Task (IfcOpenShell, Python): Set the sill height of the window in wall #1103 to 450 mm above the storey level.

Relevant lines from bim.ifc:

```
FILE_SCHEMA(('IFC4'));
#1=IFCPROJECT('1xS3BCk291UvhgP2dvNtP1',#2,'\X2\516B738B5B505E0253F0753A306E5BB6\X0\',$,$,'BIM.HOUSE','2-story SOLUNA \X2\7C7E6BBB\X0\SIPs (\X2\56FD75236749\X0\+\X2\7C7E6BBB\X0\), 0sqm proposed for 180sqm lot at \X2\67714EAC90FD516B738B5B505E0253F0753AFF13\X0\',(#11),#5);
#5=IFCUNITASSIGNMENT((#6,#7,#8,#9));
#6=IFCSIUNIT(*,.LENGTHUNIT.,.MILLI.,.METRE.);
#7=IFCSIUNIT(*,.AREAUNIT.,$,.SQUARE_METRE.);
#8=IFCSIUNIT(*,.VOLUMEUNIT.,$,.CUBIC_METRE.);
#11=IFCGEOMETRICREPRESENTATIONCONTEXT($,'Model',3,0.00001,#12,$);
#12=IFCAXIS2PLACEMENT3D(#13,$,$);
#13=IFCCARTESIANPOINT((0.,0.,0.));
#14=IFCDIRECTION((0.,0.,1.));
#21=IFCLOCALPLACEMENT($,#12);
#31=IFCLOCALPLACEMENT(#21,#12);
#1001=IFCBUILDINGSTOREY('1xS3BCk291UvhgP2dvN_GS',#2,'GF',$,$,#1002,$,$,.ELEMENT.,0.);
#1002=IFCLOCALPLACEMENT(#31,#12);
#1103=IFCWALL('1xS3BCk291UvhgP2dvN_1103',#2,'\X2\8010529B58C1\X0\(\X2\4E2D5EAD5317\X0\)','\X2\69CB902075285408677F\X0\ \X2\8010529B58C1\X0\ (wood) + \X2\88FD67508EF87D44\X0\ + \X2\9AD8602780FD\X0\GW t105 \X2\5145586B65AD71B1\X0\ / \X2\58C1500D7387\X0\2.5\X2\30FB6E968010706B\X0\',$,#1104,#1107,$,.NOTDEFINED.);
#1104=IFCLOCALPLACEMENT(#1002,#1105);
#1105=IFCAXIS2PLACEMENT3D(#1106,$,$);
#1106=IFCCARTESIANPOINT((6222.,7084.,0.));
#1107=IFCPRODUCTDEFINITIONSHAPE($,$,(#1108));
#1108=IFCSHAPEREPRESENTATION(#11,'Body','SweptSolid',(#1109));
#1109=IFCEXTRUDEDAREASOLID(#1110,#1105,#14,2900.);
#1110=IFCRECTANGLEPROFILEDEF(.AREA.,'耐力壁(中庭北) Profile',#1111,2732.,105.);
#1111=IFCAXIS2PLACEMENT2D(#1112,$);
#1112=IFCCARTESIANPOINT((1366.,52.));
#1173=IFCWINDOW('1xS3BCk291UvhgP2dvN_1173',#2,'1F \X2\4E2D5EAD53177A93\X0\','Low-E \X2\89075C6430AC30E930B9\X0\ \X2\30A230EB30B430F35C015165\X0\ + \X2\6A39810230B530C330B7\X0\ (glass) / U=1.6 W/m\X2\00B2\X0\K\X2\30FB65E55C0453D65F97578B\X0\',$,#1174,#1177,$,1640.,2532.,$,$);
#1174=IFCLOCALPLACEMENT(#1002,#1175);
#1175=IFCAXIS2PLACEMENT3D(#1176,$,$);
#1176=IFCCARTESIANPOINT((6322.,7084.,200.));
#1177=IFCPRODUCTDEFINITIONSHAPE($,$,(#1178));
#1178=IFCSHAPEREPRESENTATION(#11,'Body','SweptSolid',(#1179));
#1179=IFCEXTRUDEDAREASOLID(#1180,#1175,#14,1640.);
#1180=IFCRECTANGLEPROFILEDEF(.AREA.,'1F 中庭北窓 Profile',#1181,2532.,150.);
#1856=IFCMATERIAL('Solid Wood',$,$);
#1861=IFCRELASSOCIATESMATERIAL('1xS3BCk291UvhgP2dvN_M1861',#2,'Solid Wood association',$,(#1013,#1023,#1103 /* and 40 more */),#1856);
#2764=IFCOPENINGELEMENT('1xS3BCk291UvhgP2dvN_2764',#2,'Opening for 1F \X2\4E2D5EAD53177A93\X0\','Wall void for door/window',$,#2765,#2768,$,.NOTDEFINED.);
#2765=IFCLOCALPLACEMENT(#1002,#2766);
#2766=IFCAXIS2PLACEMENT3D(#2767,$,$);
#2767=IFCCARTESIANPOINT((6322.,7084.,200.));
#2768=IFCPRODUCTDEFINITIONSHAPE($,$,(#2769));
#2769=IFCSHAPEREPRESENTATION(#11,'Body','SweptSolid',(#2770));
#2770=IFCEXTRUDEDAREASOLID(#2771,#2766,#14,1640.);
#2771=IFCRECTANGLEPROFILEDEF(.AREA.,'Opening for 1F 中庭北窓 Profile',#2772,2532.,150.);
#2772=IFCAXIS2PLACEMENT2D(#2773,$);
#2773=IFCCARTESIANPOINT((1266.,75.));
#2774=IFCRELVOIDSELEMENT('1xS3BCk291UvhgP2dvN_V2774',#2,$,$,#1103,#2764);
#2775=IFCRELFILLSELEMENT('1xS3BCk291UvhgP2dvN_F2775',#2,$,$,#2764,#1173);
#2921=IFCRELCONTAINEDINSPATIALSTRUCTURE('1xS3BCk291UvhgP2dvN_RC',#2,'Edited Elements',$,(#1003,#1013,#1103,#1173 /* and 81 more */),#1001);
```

```python
import numpy as np
import ifcopenshell
import ifcopenshell.api.geometry
import ifcopenshell.geom
import ifcopenshell.util.element
import ifcopenshell.util.placement
import ifcopenshell.util.shape
import ifcopenshell.util.unit

model = ifcopenshell.open("bim.ifc")
unit_scale = ifcopenshell.util.unit.calculate_unit_scale(model)

window = model.by_guid("1xS3BCk291UvhgP2dvN_1173")
opening = window.FillsVoids[0].RelatingOpeningElement
storey = ifcopenshell.util.element.get_container(window, ifc_class="IfcBuildingStorey")
level = ifcopenshell.util.placement.get_local_placement(storey.ObjectPlacement)[2, 3]

# The opening's origin need not be at the sill, so measure its lowest point.
shape = ifcopenshell.geom.create_shape(ifcopenshell.geom.settings(), opening)
bottom = ifcopenshell.util.shape.get_shape_bottom_elevation(shape, shape.geometry) / unit_scale
dz = level + 0.45 / unit_scale - bottom

shift = np.array([0.0, 0.0, dz])
# The window is not placed relative to its opening, so move both.
for product in (opening, window):
    matrix = ifcopenshell.util.placement.get_local_placement(product.ObjectPlacement)
    matrix[:3, 3] += shift
    ifcopenshell.api.geometry.edit_object_placement(model, product=product, matrix=matrix, is_si=False)

print(f"moved by {dz * unit_scale:+.3f} m")

model.write("bim_edited.ifc")
```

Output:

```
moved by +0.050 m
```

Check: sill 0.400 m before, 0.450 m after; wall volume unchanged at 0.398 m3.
